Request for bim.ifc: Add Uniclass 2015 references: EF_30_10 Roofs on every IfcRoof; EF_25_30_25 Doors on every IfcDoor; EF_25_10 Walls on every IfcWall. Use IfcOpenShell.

First a look at what the model holds.

```python
import ifcopenshell

model = ifcopenshell.open("bim.ifc")
print(model.schema)
print("classifications:", [c.Name for c in model.by_type("IfcClassification")])
for ifc_class in ("IfcDoor", "IfcRoof", "IfcStair", "IfcWall", "IfcWindow"):
    print(ifc_class, len(model.by_type(ifc_class)))
```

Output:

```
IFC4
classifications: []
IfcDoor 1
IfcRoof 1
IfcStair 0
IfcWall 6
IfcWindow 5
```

```python
import ifcopenshell
import ifcopenshell.api.classification

model = ifcopenshell.open("bim.ifc")

system = ifcopenshell.api.classification.add_classification(model, classification="Uniclass 2015")

codes = {
    "IfcRoof": ("EF_30_10", "Roofs"),
    "IfcDoor": ("EF_25_30_25", "Doors"),
    "IfcWall": ("EF_25_10", "Walls"),
}
for ifc_class, (code, name) in codes.items():
    products = model.by_type(ifc_class)
    ifcopenshell.api.classification.add_reference(
        model, products=products, classification=system, identification=code, name=name
    )
    print(code, len(products))

model.write("bim_edited.ifc")
```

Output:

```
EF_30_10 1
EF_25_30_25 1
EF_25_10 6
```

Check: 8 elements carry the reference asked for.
